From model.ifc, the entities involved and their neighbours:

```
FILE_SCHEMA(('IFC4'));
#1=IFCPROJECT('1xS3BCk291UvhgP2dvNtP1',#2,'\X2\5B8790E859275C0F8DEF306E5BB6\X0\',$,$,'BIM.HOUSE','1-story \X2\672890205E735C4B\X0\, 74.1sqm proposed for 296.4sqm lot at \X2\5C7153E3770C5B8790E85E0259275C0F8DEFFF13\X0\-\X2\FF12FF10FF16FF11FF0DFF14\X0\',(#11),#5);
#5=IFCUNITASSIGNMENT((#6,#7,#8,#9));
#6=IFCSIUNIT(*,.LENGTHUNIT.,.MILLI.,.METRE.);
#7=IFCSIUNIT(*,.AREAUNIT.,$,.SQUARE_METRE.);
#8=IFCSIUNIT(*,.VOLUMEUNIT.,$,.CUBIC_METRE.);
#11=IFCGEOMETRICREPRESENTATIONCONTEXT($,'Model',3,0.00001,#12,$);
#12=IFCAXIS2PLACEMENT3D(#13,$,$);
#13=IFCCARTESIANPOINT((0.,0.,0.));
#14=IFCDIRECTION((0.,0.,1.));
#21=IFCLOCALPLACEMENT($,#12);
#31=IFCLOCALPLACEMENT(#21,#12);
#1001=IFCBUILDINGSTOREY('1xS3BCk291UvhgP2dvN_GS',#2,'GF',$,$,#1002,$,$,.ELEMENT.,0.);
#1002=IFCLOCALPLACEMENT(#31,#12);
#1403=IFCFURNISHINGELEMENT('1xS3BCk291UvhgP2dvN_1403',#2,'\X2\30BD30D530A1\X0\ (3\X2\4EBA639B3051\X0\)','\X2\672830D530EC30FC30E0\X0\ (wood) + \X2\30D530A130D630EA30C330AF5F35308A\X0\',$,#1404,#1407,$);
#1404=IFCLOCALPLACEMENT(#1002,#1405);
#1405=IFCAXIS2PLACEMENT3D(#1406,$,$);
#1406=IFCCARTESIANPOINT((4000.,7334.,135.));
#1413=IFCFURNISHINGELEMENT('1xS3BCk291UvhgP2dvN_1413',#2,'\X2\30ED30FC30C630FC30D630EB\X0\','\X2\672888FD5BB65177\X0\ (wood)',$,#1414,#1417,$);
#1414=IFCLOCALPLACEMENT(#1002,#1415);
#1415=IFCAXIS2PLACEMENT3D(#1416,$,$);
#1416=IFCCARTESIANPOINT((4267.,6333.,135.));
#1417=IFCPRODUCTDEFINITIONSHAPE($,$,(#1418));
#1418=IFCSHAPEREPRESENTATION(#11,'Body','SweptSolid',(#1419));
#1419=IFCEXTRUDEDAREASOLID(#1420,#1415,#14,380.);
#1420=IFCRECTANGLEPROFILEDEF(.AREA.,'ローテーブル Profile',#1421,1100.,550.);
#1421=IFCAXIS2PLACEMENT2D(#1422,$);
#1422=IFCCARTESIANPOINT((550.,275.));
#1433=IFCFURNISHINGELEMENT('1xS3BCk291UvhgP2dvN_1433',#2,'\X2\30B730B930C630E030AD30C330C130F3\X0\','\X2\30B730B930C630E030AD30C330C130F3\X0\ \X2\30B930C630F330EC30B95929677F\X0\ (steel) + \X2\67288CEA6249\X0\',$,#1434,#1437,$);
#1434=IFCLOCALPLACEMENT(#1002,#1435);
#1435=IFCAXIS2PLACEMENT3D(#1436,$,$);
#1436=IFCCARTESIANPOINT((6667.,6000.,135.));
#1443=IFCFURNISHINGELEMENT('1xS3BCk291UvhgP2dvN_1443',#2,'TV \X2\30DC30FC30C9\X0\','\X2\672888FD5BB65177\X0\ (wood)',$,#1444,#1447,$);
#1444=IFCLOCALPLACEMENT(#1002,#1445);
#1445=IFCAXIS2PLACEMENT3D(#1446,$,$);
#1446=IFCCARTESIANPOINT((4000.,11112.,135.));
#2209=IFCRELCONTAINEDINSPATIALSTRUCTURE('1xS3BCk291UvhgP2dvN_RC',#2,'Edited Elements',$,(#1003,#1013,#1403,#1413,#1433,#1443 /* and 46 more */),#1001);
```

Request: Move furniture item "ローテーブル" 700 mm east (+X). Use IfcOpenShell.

```python
import ifcopenshell
import ifcopenshell.api.geometry
import ifcopenshell.util.placement
import ifcopenshell.util.unit

model = ifcopenshell.open("model.ifc")
unit_scale = ifcopenshell.util.unit.calculate_unit_scale(model)

item = model.by_id(1413)
matrix = ifcopenshell.util.placement.get_local_placement(item.ObjectPlacement)
matrix[0, 3] += 0.7 / unit_scale
ifcopenshell.api.geometry.edit_object_placement(model, product=item, matrix=matrix, is_si=False)

print(ifcopenshell.util.placement.get_local_placement(item.ObjectPlacement).round(3) + 0.0)

model.write("model-out.ifc")
```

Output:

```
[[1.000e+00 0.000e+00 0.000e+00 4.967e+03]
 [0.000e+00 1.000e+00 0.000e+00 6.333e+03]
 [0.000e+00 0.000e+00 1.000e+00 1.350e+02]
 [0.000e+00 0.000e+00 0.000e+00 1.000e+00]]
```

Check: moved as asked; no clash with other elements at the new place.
